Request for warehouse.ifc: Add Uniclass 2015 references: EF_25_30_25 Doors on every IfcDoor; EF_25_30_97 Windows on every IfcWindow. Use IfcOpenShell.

First a look at what the model holds.

```python
import ifcopenshell

model = ifcopenshell.open("warehouse.ifc")
print(model.schema)
print("classifications:", [c.Name for c in model.by_type("IfcClassification")])
for ifc_class in ("IfcDoor", "IfcRoof", "IfcStair", "IfcWall", "IfcWindow"):
    print(ifc_class, len(model.by_type(ifc_class)))
```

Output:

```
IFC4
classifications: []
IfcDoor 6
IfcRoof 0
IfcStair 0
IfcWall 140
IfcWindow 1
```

```python
import ifcopenshell
import ifcopenshell.api.classification

model = ifcopenshell.open("warehouse.ifc")

system = ifcopenshell.api.classification.add_classification(model, classification="Uniclass 2015")

codes = {
    "IfcDoor": ("EF_25_30_25", "Doors"),
    "IfcWindow": ("EF_25_30_97", "Windows"),
}
for ifc_class, (code, name) in codes.items():
    products = model.by_type(ifc_class)
    ifcopenshell.api.classification.add_reference(
        model, products=products, classification=system, identification=code, name=name
    )
    print(code, len(products))

model.write("warehouse_v2.ifc")
```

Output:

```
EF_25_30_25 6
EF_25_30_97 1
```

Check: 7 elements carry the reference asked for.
